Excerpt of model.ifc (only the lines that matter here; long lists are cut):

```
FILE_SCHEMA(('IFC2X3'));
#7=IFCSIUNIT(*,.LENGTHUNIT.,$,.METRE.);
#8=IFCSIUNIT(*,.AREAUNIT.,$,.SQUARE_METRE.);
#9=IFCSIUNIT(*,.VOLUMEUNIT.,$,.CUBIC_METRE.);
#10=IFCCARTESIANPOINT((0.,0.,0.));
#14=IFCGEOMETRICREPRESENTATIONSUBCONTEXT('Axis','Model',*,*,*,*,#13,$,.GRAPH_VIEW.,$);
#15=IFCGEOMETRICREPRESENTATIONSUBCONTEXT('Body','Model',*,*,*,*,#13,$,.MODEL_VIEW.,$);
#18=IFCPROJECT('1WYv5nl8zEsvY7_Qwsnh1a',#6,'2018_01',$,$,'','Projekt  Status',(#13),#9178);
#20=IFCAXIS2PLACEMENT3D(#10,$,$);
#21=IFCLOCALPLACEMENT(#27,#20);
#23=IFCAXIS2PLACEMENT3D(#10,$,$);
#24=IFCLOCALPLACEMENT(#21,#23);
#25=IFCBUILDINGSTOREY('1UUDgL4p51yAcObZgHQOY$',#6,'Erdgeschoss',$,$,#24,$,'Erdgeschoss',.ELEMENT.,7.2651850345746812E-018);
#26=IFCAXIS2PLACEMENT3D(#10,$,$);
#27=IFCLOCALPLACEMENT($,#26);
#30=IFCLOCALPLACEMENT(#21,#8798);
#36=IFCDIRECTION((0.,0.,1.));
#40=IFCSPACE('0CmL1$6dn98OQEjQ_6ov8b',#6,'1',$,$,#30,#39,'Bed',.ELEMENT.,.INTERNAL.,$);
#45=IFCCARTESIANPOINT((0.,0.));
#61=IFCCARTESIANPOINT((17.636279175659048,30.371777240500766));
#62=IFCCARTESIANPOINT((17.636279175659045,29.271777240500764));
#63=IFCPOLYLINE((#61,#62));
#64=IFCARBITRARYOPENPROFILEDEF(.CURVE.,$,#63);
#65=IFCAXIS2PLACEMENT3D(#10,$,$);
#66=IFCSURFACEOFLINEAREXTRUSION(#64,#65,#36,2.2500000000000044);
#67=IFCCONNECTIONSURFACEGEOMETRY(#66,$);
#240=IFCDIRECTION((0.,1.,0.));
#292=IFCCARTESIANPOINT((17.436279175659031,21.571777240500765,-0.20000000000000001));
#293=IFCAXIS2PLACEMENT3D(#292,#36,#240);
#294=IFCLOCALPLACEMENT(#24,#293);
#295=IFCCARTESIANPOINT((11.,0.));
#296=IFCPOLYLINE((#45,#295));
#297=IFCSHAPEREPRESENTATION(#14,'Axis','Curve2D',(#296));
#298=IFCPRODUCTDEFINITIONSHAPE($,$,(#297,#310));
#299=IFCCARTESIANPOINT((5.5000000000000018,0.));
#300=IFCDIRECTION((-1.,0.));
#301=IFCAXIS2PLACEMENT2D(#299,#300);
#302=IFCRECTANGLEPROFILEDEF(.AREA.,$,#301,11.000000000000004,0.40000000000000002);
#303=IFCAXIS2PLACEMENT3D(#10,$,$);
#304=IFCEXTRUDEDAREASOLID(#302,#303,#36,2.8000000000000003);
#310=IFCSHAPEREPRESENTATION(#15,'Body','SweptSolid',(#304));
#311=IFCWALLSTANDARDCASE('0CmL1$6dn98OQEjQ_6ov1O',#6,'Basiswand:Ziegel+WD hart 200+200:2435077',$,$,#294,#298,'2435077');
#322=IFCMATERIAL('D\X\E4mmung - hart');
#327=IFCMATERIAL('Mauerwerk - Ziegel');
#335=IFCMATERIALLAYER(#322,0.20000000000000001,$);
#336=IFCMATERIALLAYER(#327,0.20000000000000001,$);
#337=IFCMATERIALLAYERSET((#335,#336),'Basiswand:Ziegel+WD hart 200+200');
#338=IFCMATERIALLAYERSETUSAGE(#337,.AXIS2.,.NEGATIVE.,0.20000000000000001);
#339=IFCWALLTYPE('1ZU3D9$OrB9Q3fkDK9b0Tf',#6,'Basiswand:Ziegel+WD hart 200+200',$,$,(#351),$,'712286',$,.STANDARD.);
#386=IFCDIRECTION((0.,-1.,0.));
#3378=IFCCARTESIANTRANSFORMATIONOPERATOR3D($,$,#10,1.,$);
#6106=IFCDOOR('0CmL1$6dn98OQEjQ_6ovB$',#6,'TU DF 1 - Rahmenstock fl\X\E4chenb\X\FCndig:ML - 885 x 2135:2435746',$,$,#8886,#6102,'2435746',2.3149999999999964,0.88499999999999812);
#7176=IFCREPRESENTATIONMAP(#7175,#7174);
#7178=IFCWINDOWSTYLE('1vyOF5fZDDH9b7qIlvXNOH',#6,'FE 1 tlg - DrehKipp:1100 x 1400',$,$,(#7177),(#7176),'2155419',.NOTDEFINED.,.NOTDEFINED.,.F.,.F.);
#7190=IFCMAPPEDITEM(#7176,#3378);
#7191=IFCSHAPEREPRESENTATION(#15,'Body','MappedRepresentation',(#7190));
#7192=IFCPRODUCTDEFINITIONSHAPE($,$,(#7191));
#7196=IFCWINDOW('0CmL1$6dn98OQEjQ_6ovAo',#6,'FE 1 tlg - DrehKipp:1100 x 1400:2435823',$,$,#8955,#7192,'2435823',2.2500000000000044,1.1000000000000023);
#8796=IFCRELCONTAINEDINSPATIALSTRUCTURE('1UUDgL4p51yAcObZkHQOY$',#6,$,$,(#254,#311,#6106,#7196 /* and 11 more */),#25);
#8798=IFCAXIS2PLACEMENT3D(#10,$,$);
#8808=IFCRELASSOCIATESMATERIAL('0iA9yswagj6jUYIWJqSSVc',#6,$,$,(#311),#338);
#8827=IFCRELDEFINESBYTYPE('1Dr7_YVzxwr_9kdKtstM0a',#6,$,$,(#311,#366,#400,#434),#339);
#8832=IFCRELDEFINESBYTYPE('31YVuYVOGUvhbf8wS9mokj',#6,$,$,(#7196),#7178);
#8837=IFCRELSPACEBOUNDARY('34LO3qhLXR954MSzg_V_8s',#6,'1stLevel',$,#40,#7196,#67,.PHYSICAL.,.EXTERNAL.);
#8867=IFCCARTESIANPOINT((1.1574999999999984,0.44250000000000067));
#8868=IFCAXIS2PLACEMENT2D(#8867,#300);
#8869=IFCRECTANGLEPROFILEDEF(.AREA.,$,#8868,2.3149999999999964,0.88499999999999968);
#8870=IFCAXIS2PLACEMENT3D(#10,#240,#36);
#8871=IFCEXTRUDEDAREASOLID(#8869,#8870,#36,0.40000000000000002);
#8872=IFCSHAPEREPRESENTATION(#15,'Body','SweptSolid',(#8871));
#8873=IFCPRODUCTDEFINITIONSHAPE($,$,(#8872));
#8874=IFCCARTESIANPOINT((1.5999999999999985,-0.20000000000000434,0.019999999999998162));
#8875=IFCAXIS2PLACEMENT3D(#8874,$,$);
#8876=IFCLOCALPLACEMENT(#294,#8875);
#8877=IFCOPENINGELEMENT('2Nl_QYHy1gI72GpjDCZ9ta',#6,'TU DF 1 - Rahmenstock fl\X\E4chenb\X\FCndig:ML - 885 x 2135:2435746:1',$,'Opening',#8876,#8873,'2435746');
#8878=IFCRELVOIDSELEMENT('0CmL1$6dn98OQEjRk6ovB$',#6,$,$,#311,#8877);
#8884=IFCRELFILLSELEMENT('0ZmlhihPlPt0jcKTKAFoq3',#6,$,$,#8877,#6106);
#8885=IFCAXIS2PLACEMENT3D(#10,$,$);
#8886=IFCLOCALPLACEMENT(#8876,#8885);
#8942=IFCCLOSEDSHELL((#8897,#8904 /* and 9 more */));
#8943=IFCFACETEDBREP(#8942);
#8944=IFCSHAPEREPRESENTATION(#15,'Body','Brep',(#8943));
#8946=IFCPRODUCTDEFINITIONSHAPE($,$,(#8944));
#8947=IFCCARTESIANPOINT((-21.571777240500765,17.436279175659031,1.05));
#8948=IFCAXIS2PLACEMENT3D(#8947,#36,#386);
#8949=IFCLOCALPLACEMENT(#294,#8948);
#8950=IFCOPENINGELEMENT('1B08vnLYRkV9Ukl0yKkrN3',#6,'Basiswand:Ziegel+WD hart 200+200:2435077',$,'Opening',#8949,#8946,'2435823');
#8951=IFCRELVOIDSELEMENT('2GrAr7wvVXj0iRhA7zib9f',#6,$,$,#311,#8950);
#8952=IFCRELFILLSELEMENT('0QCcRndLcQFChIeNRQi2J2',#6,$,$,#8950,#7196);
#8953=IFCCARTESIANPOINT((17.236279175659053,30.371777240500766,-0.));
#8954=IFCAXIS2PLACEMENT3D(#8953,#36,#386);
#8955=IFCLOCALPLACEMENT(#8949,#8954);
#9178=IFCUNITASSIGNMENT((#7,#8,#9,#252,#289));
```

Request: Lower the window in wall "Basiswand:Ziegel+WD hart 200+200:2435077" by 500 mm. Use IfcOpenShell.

```python
import numpy as np
import ifcopenshell
import ifcopenshell.api.geometry
import ifcopenshell.util.placement
import ifcopenshell.util.unit

model = ifcopenshell.open("model.ifc")
unit_scale = ifcopenshell.util.unit.calculate_unit_scale(model)

window = model.by_guid("0CmL1$6dn98OQEjQ_6ovAo")
opening = window.FillsVoids[0].RelatingOpeningElement
dz = -0.5

shift = np.array([0.0, 0.0, dz])
# The window is placed relative to its opening, so it follows when the opening moves.
matrix = ifcopenshell.util.placement.get_local_placement(opening.ObjectPlacement)
matrix[:3, 3] += shift
ifcopenshell.api.geometry.edit_object_placement(
    model, product=opening, matrix=matrix, is_si=False, should_transform_children=True
)

# Space boundary surfaces are stored in each space's coordinates; move them too.
for rel in window.ProvidesBoundaries:
    if not rel.ConnectionGeometry:
        continue
    surface = rel.ConnectionGeometry.SurfaceOnRelatingElement
    space_matrix = ifcopenshell.util.placement.get_local_placement(rel.RelatingSpace.ObjectPlacement)
    point = np.array(surface.Position.Location.Coordinates) + space_matrix[:3, :3].T @ shift
    surface.Position = model.createIfcAxis2Placement3D(
        model.createIfcCartesianPoint(point.tolist()), surface.Position.Axis, surface.Position.RefDirection
    )

print(f"moved by {dz * unit_scale:+.3f} m")

model.write("model-out.ifc")
```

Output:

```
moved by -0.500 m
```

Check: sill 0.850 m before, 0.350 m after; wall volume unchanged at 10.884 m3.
